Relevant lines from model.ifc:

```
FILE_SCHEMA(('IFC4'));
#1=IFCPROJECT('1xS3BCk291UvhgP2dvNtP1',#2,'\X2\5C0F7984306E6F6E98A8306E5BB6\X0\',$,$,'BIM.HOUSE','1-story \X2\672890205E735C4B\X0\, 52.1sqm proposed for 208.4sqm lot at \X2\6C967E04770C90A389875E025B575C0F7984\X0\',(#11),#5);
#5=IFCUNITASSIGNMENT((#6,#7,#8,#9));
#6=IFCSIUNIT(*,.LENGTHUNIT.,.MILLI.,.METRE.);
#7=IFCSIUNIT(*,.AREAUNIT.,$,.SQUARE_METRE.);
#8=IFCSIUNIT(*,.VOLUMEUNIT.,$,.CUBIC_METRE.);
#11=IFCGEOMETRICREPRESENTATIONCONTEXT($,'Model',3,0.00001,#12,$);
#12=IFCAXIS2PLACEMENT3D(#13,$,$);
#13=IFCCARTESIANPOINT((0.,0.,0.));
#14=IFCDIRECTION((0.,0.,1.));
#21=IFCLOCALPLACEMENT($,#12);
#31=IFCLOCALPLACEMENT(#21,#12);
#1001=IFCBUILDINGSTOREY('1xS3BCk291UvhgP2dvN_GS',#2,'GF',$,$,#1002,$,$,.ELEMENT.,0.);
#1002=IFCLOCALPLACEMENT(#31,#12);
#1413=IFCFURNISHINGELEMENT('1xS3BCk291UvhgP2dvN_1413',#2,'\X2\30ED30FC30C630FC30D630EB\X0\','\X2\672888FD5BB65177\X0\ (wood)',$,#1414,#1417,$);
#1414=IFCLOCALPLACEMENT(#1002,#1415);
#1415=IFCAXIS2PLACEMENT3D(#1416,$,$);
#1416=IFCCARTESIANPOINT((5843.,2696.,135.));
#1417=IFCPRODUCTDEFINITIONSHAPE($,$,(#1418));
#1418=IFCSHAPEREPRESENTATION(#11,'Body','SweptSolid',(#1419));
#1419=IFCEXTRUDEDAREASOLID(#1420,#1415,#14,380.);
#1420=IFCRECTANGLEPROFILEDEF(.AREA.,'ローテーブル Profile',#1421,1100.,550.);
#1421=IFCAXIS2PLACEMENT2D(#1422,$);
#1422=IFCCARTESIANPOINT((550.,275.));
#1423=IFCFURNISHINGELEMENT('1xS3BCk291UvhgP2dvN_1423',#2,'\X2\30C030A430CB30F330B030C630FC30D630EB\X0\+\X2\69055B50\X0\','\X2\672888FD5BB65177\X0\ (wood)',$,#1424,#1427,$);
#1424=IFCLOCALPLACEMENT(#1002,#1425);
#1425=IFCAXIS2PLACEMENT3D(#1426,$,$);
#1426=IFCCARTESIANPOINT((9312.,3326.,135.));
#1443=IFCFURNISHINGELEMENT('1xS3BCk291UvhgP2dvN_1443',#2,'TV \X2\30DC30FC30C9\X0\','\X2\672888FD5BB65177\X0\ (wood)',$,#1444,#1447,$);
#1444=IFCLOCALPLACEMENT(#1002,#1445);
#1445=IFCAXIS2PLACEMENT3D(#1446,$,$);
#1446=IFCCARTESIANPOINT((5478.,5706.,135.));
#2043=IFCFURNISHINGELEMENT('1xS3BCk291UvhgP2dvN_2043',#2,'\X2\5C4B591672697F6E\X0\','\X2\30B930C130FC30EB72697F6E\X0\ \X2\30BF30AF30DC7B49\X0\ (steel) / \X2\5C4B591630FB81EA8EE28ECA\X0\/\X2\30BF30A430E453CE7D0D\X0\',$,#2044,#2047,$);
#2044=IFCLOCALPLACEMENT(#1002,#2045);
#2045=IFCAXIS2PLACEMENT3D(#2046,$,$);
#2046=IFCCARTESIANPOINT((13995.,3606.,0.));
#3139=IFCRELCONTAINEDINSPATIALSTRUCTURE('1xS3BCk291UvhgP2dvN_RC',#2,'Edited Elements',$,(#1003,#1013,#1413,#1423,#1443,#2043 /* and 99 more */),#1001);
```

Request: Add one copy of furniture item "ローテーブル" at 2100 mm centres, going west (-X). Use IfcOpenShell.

```python
import numpy as np
import ifcopenshell
import ifcopenshell.api.geometry
import ifcopenshell.api.root
import ifcopenshell.util.element
import ifcopenshell.util.placement
import ifcopenshell.util.unit

model = ifcopenshell.open("model.ifc")
unit_scale = ifcopenshell.util.unit.calculate_unit_scale(model)


def reuse_history(source, copy):
    """copy_class also copies each property set's owner history, people and application; keep the originals."""
    for rel in copy.IsDefinedBy:
        if rel.is_a("IfcRelDefinesByProperties") and (history := rel.RelatingPropertyDefinition.OwnerHistory):
            rel.RelatingPropertyDefinition.OwnerHistory = source.OwnerHistory
            ifcopenshell.util.element.remove_deep2(model, history)


source = model.by_guid("1xS3BCk291UvhgP2dvN_1413")
base = ifcopenshell.util.placement.get_local_placement(source.ObjectPlacement)
step = np.array([-1.0, 0.0, 0.0]) * 2.1 / unit_scale

for i in range(1, 2):
    copy = ifcopenshell.api.root.copy_class(model, product=source)
    copy.Representation = ifcopenshell.util.element.copy_deep(
        model, source.Representation, exclude=["IfcGeometricRepresentationContext", "IfcRepresentationMap"]
    )
    reuse_history(source, copy)
    matrix = base.copy()
    matrix[:3, 3] += i * step
    print("added at", matrix[:3, 3].round(3) + 0.0)
    ifcopenshell.api.geometry.edit_object_placement(model, product=copy, matrix=matrix, is_si=False)

model.write("model-out.ifc")
```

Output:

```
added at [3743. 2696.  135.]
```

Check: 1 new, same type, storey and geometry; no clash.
